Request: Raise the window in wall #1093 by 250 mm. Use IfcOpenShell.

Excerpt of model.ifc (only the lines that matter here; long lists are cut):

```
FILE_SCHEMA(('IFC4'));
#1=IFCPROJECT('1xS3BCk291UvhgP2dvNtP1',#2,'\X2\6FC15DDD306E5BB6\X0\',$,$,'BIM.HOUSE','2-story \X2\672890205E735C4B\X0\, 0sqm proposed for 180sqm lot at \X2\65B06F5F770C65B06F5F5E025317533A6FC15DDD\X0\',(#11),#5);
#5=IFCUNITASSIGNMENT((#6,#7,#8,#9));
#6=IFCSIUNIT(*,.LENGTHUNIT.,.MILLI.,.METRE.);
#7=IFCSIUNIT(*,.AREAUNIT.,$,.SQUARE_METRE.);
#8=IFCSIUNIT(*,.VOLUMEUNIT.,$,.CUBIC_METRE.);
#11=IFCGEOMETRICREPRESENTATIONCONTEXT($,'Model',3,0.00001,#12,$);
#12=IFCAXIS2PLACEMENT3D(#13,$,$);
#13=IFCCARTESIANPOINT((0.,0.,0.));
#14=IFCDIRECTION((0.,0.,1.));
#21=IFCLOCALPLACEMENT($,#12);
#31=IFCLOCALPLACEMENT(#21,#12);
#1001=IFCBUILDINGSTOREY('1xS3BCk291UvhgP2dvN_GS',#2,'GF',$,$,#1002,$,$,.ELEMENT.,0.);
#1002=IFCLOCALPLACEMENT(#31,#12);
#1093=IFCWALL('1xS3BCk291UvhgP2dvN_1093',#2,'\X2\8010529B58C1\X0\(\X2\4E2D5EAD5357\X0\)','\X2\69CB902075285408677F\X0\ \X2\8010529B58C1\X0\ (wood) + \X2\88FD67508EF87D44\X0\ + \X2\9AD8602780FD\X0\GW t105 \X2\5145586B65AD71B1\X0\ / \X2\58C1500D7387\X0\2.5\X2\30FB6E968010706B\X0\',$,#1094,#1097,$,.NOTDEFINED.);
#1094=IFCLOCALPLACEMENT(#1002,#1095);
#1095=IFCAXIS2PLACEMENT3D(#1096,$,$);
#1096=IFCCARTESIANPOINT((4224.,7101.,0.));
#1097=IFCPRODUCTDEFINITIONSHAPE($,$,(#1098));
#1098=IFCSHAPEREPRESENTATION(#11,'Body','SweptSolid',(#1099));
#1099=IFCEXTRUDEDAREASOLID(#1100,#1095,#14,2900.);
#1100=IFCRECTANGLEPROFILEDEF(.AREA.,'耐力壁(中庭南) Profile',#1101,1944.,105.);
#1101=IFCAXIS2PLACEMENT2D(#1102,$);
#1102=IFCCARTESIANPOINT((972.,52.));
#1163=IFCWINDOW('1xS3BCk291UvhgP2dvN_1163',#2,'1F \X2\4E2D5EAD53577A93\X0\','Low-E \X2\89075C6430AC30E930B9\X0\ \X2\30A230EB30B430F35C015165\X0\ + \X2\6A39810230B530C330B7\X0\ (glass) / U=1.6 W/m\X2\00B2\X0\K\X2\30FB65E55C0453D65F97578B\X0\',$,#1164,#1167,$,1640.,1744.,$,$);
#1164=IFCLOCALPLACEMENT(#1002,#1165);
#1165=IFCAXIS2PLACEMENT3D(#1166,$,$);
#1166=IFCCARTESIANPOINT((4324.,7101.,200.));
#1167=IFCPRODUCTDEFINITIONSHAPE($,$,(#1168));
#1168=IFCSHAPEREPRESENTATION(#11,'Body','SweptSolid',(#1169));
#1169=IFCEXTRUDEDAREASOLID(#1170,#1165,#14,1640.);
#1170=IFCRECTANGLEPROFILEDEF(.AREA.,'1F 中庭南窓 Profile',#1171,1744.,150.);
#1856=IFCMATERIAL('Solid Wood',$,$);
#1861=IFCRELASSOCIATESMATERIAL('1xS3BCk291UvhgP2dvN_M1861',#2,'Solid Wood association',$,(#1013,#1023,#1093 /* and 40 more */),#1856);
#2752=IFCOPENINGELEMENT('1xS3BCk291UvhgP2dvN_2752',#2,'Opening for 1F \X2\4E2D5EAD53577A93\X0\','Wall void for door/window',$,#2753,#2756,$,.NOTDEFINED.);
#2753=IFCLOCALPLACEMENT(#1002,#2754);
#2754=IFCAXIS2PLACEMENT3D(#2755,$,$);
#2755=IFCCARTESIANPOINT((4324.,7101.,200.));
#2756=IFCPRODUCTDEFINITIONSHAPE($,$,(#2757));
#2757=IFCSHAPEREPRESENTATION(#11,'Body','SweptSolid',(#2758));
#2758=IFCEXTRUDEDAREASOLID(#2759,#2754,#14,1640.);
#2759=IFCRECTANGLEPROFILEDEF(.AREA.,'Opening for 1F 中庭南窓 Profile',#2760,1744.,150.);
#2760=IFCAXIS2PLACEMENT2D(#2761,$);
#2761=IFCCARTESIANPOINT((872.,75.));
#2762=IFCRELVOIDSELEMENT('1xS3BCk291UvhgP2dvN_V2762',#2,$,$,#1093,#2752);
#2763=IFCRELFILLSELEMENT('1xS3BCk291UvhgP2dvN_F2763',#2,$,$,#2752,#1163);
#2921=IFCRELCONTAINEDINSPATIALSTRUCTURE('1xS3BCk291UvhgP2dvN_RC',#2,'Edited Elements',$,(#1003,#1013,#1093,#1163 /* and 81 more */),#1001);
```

```python
import numpy as np
import ifcopenshell
import ifcopenshell.api.geometry
import ifcopenshell.util.placement
import ifcopenshell.util.unit

model = ifcopenshell.open("model.ifc")
unit_scale = ifcopenshell.util.unit.calculate_unit_scale(model)

window = model.by_guid("1xS3BCk291UvhgP2dvN_1163")
opening = window.FillsVoids[0].RelatingOpeningElement
dz = 0.25 / unit_scale

shift = np.array([0.0, 0.0, dz])
# The window is not placed relative to its opening, so move both.
for product in (opening, window):
    matrix = ifcopenshell.util.placement.get_local_placement(product.ObjectPlacement)
    matrix[:3, 3] += shift
    ifcopenshell.api.geometry.edit_object_placement(model, product=product, matrix=matrix, is_si=False)

print(f"moved by {dz * unit_scale:+.3f} m")

model.write("model_updated.ifc")
```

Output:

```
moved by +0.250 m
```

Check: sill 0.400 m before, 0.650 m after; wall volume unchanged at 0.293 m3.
